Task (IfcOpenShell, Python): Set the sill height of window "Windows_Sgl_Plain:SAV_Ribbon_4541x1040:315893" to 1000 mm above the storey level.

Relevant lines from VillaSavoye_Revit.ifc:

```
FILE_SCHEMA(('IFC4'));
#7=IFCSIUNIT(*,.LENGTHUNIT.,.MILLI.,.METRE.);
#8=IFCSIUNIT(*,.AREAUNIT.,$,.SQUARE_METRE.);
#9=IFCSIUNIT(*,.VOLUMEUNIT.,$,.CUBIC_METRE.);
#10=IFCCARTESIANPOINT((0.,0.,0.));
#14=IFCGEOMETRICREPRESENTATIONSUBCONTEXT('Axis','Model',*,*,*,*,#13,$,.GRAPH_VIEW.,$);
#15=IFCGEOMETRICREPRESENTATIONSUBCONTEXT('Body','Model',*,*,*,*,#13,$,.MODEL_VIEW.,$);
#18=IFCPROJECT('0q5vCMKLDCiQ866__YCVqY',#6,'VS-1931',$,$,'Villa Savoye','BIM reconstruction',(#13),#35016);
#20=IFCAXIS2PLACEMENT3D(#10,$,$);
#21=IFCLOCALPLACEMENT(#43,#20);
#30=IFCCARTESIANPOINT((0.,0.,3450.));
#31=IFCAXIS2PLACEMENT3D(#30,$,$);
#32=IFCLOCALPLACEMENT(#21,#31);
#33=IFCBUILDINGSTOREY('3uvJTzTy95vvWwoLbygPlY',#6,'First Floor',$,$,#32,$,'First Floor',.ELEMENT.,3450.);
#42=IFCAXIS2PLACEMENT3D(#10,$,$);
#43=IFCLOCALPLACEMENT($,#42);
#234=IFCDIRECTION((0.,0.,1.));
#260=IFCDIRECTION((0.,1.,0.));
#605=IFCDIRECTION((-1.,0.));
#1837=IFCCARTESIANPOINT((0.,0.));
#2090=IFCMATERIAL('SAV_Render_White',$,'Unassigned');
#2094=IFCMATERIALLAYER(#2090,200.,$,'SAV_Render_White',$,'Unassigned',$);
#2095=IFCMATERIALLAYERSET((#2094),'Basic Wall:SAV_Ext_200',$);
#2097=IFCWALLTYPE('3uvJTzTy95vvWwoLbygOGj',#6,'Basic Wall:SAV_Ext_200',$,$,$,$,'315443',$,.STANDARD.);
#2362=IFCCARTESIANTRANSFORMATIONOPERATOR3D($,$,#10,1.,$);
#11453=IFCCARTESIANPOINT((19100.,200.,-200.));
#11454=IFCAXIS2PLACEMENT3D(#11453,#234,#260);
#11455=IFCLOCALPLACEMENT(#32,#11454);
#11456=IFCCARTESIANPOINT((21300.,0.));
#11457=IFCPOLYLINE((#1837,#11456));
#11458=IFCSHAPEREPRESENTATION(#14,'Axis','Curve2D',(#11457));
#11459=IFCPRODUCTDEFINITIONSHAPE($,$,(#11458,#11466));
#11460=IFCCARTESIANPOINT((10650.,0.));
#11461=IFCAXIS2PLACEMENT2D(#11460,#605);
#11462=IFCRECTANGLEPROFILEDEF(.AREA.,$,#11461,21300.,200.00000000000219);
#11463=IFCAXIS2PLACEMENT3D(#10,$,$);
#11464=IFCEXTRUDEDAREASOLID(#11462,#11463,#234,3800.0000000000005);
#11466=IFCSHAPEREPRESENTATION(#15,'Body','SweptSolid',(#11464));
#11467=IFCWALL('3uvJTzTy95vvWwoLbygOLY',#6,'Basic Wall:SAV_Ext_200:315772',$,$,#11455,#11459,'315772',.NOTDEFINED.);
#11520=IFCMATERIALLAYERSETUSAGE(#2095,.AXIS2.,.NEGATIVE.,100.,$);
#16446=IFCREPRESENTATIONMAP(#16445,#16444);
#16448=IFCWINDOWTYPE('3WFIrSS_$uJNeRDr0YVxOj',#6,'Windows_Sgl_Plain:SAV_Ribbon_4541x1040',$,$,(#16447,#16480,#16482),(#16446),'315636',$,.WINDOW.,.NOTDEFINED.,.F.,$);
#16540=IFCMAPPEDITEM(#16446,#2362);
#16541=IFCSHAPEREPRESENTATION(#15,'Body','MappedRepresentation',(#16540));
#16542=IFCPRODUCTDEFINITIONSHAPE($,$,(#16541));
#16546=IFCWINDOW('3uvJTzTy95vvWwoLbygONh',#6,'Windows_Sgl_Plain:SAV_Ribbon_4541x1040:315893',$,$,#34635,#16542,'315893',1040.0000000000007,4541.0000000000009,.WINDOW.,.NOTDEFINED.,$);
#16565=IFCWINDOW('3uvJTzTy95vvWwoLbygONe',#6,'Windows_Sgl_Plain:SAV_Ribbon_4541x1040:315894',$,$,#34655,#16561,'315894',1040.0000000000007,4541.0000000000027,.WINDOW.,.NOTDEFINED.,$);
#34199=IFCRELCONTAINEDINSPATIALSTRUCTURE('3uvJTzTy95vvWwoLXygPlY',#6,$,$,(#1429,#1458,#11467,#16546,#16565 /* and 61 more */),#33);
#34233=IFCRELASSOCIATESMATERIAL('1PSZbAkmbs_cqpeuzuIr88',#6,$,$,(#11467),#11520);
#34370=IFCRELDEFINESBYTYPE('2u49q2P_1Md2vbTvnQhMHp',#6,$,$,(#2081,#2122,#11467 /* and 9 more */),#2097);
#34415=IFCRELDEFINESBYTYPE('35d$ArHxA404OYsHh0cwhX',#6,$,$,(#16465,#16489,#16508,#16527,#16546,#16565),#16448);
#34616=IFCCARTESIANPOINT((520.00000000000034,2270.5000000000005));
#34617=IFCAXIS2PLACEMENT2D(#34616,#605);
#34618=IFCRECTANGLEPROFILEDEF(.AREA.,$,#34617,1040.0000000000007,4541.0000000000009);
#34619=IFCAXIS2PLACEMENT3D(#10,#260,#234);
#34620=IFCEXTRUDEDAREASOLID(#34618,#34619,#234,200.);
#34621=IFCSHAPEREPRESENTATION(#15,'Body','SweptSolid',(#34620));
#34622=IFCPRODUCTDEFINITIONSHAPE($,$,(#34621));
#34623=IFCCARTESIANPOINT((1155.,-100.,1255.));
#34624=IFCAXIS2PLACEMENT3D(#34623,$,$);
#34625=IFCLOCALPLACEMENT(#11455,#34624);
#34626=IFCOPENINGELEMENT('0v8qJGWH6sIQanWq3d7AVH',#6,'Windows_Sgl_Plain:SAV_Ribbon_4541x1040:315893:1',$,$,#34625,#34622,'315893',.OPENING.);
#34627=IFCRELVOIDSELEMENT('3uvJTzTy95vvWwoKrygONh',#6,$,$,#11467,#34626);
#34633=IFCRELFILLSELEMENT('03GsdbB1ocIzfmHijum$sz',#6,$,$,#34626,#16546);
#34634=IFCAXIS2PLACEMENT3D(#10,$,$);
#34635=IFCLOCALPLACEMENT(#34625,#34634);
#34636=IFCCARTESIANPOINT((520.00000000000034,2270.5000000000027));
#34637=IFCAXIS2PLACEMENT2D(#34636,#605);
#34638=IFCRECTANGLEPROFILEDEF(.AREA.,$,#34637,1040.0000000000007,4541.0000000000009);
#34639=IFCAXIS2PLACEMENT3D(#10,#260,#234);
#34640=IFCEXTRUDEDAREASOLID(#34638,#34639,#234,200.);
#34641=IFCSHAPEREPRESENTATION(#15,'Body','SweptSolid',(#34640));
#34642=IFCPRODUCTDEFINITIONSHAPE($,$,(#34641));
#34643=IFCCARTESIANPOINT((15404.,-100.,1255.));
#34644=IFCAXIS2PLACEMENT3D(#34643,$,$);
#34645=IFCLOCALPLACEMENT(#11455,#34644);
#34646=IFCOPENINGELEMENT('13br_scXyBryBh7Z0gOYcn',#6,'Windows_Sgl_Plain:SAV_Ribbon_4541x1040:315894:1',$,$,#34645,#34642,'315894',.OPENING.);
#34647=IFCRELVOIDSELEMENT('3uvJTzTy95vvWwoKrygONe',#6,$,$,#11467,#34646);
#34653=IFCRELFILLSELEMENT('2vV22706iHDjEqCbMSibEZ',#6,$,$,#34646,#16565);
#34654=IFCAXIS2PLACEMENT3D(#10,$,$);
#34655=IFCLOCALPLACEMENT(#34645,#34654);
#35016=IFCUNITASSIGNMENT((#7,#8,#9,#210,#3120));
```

```python
import numpy as np
import ifcopenshell
import ifcopenshell.api.geometry
import ifcopenshell.geom
import ifcopenshell.util.element
import ifcopenshell.util.placement
import ifcopenshell.util.shape
import ifcopenshell.util.unit

model = ifcopenshell.open("VillaSavoye_Revit.ifc")
unit_scale = ifcopenshell.util.unit.calculate_unit_scale(model)

window = model.by_guid("3uvJTzTy95vvWwoLbygONh")
opening = window.FillsVoids[0].RelatingOpeningElement
storey = ifcopenshell.util.element.get_container(window, ifc_class="IfcBuildingStorey")
level = ifcopenshell.util.placement.get_local_placement(storey.ObjectPlacement)[2, 3]

# The opening's origin need not be at the sill, so measure its lowest point.
shape = ifcopenshell.geom.create_shape(ifcopenshell.geom.settings(), opening)
bottom = ifcopenshell.util.shape.get_shape_bottom_elevation(shape, shape.geometry) / unit_scale
dz = level + 1 / unit_scale - bottom

shift = np.array([0.0, 0.0, dz])
# The window is placed relative to its opening, so it follows when the opening moves.
matrix = ifcopenshell.util.placement.get_local_placement(opening.ObjectPlacement)
matrix[:3, 3] += shift
ifcopenshell.api.geometry.edit_object_placement(
    model, product=opening, matrix=matrix, is_si=False, should_transform_children=True
)

print(f"moved by {dz * unit_scale:+.3f} m")

model.write("VillaSavoye_Revit_updated.ifc")
```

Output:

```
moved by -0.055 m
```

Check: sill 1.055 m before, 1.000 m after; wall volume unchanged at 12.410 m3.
